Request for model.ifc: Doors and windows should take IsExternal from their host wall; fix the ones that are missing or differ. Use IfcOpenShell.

First a look at what the model holds.

```python
import ifcopenshell
import ifcopenshell.util.element

model = ifcopenshell.open("model.ifc")
print(model.schema)
seen = {}
for e in model.by_type("IfcDoor") + model.by_type("IfcWindow"):
    if not e.FillsVoids:
        continue
    host = e.FillsVoids[0].RelatingOpeningElement.VoidsElements[0].RelatingBuildingElement
    own = ifcopenshell.util.element.get_pset(e, f"Pset_{e.is_a()[3:].removesuffix('StandardCase')}Common", "IsExternal")
    wall = ifcopenshell.util.element.get_pset(host, "Pset_WallCommon", "IsExternal")
    seen[e.is_a(), own, wall] = seen.get((e.is_a(), own, wall), 0) + 1
for (cls, own, wall), count in sorted(seen.items(), key=str):
    print(count, cls, "IsExternal:", own, "| host wall:", wall)
```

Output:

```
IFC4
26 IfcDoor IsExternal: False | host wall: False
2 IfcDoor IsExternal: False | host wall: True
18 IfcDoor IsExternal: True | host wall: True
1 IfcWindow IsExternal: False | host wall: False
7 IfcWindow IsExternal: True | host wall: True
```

```python
import ifcopenshell
import ifcopenshell.api.pset
import ifcopenshell.util.element

model = ifcopenshell.open("model.ifc")

count = 0
for ifc_class, pset_name in (("IfcDoor", "Pset_DoorCommon"), ("IfcWindow", "Pset_WindowCommon")):
    for e in model.by_type(ifc_class):
        if not e.FillsVoids:
            continue
        host = e.FillsVoids[0].RelatingOpeningElement.VoidsElements[0].RelatingBuildingElement
        external = ifcopenshell.util.element.get_pset(host, "Pset_WallCommon", "IsExternal")
        if external is None or ifcopenshell.util.element.get_pset(e, pset_name, "IsExternal") == external:
            continue
        pset = ifcopenshell.api.pset.add_pset(model, product=e, name=pset_name)
        ifcopenshell.api.pset.edit_pset(model, pset=pset, properties={"IsExternal": external})
        count += 1

print(count, "updated")

model.write("model_v2.ifc")
```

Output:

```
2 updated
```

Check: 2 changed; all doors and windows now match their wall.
